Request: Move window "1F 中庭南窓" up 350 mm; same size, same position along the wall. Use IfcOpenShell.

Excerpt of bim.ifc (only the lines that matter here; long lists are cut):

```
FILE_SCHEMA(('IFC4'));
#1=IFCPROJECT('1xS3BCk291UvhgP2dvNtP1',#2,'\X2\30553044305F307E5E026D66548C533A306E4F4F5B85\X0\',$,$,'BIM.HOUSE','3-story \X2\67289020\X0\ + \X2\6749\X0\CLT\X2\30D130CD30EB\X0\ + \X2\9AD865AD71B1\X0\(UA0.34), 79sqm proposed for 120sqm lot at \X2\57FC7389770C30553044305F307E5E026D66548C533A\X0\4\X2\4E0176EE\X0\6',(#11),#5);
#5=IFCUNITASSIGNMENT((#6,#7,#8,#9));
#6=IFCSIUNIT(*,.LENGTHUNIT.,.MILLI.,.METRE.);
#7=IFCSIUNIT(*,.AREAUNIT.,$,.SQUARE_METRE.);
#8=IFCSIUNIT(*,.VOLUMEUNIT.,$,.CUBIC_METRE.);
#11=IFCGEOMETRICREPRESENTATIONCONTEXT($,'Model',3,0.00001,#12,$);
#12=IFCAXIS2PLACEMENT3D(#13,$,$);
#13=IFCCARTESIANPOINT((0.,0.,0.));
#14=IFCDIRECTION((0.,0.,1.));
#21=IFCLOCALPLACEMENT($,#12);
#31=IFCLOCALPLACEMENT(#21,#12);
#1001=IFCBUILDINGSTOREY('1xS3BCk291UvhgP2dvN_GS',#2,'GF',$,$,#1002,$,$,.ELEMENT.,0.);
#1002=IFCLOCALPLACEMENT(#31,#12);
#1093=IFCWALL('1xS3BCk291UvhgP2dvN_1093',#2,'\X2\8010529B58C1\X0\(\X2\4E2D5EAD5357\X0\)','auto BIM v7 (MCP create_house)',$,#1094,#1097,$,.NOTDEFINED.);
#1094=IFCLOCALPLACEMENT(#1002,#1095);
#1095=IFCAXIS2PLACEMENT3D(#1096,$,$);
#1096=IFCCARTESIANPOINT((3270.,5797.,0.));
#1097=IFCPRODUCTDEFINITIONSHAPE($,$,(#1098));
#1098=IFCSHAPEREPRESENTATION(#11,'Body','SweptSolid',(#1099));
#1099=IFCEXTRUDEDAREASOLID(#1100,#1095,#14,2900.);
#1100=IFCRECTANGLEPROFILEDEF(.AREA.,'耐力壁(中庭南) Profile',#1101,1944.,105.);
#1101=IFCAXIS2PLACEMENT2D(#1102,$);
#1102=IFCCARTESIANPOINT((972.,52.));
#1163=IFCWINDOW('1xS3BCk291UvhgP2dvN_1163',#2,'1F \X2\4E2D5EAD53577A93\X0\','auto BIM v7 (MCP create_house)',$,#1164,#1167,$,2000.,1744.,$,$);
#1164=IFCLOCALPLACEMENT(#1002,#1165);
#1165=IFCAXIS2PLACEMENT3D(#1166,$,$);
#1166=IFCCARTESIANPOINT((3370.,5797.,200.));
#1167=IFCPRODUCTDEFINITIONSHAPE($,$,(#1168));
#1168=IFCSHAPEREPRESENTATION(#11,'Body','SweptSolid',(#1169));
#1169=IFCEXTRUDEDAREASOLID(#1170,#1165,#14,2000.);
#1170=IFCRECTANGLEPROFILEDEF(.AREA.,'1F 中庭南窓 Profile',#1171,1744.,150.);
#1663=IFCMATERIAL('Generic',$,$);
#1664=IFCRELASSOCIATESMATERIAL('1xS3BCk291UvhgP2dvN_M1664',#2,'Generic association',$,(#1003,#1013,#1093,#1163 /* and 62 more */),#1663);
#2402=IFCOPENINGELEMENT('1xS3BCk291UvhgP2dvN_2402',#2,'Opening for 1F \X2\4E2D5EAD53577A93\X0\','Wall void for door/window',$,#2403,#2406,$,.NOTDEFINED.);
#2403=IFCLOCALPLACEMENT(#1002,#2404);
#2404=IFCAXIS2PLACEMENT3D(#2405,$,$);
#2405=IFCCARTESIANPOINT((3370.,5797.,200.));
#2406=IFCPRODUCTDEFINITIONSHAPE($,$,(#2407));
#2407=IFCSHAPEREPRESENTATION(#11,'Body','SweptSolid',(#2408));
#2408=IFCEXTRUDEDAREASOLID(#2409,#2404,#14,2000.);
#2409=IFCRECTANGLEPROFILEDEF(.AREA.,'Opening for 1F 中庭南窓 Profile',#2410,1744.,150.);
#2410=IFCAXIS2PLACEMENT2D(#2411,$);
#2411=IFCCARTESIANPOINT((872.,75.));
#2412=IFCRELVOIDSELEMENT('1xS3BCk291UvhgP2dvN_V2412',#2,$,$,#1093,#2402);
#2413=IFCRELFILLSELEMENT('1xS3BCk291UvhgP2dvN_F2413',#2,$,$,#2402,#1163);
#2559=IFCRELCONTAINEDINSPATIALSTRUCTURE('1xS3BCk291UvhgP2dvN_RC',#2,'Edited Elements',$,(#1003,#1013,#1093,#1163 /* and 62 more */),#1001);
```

```python
import numpy as np
import ifcopenshell
import ifcopenshell.api.geometry
import ifcopenshell.util.placement
import ifcopenshell.util.unit

model = ifcopenshell.open("bim.ifc")
unit_scale = ifcopenshell.util.unit.calculate_unit_scale(model)

window = model.by_guid("1xS3BCk291UvhgP2dvN_1163")
opening = window.FillsVoids[0].RelatingOpeningElement
dz = 350.0

shift = np.array([0.0, 0.0, dz])
# The window is not placed relative to its opening, so move both.
for product in (opening, window):
    matrix = ifcopenshell.util.placement.get_local_placement(product.ObjectPlacement)
    matrix[:3, 3] += shift
    ifcopenshell.api.geometry.edit_object_placement(model, product=product, matrix=matrix, is_si=False)

print(f"moved by {dz * unit_scale:+.3f} m")

model.write("bim_updated.ifc")
```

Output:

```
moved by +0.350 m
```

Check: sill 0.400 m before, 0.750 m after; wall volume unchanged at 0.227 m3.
